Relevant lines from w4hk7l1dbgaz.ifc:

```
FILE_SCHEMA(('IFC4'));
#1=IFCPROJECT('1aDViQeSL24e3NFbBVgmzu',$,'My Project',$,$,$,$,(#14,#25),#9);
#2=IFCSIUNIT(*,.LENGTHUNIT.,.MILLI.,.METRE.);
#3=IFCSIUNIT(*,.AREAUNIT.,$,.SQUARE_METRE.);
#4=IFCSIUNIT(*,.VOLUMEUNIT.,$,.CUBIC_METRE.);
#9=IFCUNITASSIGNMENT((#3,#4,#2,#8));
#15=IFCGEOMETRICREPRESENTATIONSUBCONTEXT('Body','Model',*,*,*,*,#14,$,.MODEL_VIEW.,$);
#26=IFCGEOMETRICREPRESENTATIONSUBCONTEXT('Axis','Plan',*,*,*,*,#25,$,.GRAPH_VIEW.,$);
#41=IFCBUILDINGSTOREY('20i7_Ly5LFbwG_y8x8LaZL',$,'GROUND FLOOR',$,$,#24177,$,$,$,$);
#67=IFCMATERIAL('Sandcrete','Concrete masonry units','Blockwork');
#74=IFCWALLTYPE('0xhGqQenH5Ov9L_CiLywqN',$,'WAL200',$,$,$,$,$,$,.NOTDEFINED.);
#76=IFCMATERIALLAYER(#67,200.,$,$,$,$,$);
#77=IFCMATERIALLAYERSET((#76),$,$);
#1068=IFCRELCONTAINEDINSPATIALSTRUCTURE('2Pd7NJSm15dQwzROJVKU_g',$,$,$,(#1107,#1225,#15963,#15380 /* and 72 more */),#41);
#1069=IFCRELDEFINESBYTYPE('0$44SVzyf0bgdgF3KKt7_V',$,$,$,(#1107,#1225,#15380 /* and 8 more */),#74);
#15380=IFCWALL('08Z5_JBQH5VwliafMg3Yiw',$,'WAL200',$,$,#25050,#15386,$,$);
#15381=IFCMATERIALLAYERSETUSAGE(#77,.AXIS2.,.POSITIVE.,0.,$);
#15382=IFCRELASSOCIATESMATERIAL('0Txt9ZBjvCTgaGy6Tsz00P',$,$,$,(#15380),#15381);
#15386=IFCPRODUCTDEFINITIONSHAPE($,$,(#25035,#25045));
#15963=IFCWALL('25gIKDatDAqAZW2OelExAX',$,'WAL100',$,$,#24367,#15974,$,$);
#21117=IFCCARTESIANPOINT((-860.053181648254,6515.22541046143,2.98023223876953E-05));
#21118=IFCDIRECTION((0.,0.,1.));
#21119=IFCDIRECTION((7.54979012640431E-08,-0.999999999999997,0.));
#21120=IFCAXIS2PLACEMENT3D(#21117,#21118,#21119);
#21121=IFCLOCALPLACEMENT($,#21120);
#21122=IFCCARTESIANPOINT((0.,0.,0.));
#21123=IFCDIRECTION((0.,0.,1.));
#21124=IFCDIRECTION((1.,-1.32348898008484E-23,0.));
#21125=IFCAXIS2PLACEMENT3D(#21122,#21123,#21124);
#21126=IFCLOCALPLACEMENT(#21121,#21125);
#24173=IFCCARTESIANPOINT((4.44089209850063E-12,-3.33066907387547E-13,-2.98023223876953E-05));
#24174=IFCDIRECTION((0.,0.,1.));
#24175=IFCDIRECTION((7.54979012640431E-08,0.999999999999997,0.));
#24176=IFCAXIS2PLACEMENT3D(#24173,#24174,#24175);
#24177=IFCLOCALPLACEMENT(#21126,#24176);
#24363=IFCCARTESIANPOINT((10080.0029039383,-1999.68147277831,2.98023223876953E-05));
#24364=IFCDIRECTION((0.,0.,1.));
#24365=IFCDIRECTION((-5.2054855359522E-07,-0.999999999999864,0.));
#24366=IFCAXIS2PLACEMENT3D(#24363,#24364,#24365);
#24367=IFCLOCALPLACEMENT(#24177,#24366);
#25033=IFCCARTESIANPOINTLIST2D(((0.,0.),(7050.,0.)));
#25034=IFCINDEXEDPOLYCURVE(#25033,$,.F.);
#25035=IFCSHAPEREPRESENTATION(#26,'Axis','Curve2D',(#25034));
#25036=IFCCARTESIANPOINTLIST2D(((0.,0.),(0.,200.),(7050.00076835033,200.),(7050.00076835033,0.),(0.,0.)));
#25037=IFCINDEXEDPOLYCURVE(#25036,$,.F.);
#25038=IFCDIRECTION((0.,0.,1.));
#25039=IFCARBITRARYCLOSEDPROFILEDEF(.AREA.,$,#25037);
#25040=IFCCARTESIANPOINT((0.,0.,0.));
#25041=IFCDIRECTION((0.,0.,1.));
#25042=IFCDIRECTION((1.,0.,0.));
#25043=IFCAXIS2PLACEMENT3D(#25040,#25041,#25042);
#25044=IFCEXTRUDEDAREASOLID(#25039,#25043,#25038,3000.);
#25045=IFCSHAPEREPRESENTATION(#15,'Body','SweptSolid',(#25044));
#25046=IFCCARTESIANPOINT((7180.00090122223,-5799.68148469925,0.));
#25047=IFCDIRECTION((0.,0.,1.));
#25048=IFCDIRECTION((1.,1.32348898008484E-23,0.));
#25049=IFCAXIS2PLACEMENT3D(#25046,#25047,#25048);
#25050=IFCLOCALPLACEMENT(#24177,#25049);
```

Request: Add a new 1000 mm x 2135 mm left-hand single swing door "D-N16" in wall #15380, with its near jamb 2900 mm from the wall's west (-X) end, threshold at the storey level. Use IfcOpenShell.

```python
import numpy as np
import ifcopenshell
import ifcopenshell.api.feature
import ifcopenshell.api.geometry
import ifcopenshell.api.root
import ifcopenshell.api.spatial
import ifcopenshell.geom
import ifcopenshell.util.element
import ifcopenshell.util.placement
import ifcopenshell.util.representation
import ifcopenshell.util.shape
import ifcopenshell.util.unit

model = ifcopenshell.open("w4hk7l1dbgaz.ifc")
unit_scale = ifcopenshell.util.unit.calculate_unit_scale(model)
settings = ifcopenshell.geom.settings()


def volume(element):
    """Net volume in cubic metres, openings subtracted."""
    shape = ifcopenshell.geom.create_shape(settings, element)
    return ifcopenshell.util.shape.get_volume(shape.geometry)


wall = model.by_guid("08Z5_JBQH5VwliafMg3Yiw")
storey = ifcopenshell.util.element.get_container(wall, ifc_class="IfcBuildingStorey")
context = ifcopenshell.util.representation.get_context(model, "Model", "Body", "MODEL_VIEW")
before = volume(wall)

width, height, from_end, sill = 1, 2.135, 2.9, 0.0  # metres

# The wall runs along its own X axis, and the end named is its -X end.
wall_shape = ifcopenshell.geom.create_shape(settings, wall)
x, y, z = ifcopenshell.util.shape.get_vertices(wall_shape.geometry).T
start = x.min() + from_end
face, thickness = float(y.min()), float(y.max() - y.min())
wall_matrix = ifcopenshell.util.placement.get_local_placement(wall.ObjectPlacement)
level = ifcopenshell.util.placement.get_local_placement(storey.ObjectPlacement)[2, 3]


def in_wall(x, y):
    """Placement at x, y metres in the wall's axes, at sill height."""
    matrix = wall_matrix.copy()
    matrix[:, 3] = wall_matrix @ np.array([x / unit_scale, y / unit_scale, 0.0, 1.0])
    matrix[2, 3] = level + sill / unit_scale
    return matrix


# Opening: a box that overshoots both wall faces by 50 mm.
opening = ifcopenshell.api.root.create_entity(model, ifc_class="IfcOpeningElement", predefined_type="OPENING")
box = ifcopenshell.api.geometry.add_wall_representation(
    model, context=context, length=width, height=height, thickness=thickness + 0.1
)
ifcopenshell.api.geometry.assign_representation(model, product=opening, representation=box)
ifcopenshell.api.geometry.edit_object_placement(model, product=opening, matrix=in_wall(start, face - 0.05), is_si=False)
ifcopenshell.api.feature.add_feature(model, feature=opening, element=wall)

door = ifcopenshell.api.root.create_entity(model, ifc_class="IfcDoor", name="D-N16", predefined_type="DOOR")
door.OverallWidth, door.OverallHeight = width / unit_scale, height / unit_scale
door.OperationType = "SINGLE_SWING_LEFT"
body = ifcopenshell.api.geometry.add_door_representation(
    model,
    context=context,
    overall_width=door.OverallWidth,
    overall_height=door.OverallHeight,
    operation_type="SINGLE_SWING_LEFT",
    lining_properties={"LiningDepth": thickness / unit_scale, "ThresholdDepth": thickness / unit_scale},
)
ifcopenshell.api.geometry.assign_representation(model, product=door, representation=body)
ifcopenshell.api.spatial.assign_container(model, products=[door], relating_structure=storey)
ifcopenshell.api.feature.add_filling(model, opening=opening, element=door)

# The lining spans the wall, so the door starts at the wall face.
ifcopenshell.api.geometry.edit_object_placement(model, product=door, matrix=in_wall(start, face), is_si=False)

after = volume(wall)

print(f"wall volume {before:.3f} -> {after:.3f} m3")

model.write("w4hk7l1dbgaz_updated.ifc")
```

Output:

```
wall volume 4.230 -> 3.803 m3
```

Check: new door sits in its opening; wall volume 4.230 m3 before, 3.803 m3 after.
